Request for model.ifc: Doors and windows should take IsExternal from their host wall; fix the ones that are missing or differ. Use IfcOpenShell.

First a look at what the model holds.

```python
import ifcopenshell
import ifcopenshell.util.element

model = ifcopenshell.open("model.ifc")
print(model.schema)
seen = {}
for e in model.by_type("IfcDoor") + model.by_type("IfcWindow"):
    if not e.FillsVoids:
        continue
    host = e.FillsVoids[0].RelatingOpeningElement.VoidsElements[0].RelatingBuildingElement
    own = ifcopenshell.util.element.get_pset(e, f"Pset_{e.is_a()[3:].removesuffix('StandardCase')}Common", "IsExternal")
    wall = ifcopenshell.util.element.get_pset(host, "Pset_WallCommon", "IsExternal")
    seen[e.is_a(), own, wall] = seen.get((e.is_a(), own, wall), 0) + 1
for (cls, own, wall), count in sorted(seen.items(), key=str):
    print(count, cls, "IsExternal:", own, "| host wall:", wall)
```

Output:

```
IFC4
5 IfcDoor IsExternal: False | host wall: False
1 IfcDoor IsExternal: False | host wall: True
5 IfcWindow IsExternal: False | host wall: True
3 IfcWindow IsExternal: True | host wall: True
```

```python
import ifcopenshell
import ifcopenshell.api.pset
import ifcopenshell.util.element

model = ifcopenshell.open("model.ifc")

count = 0
for ifc_class, pset_name in (("IfcDoor", "Pset_DoorCommon"), ("IfcWindow", "Pset_WindowCommon")):
    for e in model.by_type(ifc_class):
        if not e.FillsVoids:
            continue
        host = e.FillsVoids[0].RelatingOpeningElement.VoidsElements[0].RelatingBuildingElement
        external = ifcopenshell.util.element.get_pset(host, "Pset_WallCommon", "IsExternal")
        if external is None or ifcopenshell.util.element.get_pset(e, pset_name, "IsExternal") == external:
            continue
        pset = ifcopenshell.api.pset.add_pset(model, product=e, name=pset_name)
        ifcopenshell.api.pset.edit_pset(model, pset=pset, properties={"IsExternal": external})
        count += 1

print(count, "updated")

model.write("model_rev.ifc")
```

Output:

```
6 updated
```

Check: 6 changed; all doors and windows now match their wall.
